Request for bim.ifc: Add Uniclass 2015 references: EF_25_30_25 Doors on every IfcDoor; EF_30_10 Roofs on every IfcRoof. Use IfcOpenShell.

First a look at what the model holds.

```python
import ifcopenshell

model = ifcopenshell.open("bim.ifc")
print(model.schema)
print("classifications:", [c.Name for c in model.by_type("IfcClassification")])
for ifc_class in ("IfcDoor", "IfcRoof", "IfcStair", "IfcWall", "IfcWindow"):
    print(ifc_class, len(model.by_type(ifc_class)))
```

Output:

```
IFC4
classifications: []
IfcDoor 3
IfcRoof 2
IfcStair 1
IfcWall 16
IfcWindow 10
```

```python
import ifcopenshell
import ifcopenshell.api.classification

model = ifcopenshell.open("bim.ifc")

system = ifcopenshell.api.classification.add_classification(model, classification="Uniclass 2015")

codes = {
    "IfcDoor": ("EF_25_30_25", "Doors"),
    "IfcRoof": ("EF_30_10", "Roofs"),
}
for ifc_class, (code, name) in codes.items():
    products = model.by_type(ifc_class)
    ifcopenshell.api.classification.add_reference(
        model, products=products, classification=system, identification=code, name=name
    )
    print(code, len(products))

model.write("bim_v2.ifc")
```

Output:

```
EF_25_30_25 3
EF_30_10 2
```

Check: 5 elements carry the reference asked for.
